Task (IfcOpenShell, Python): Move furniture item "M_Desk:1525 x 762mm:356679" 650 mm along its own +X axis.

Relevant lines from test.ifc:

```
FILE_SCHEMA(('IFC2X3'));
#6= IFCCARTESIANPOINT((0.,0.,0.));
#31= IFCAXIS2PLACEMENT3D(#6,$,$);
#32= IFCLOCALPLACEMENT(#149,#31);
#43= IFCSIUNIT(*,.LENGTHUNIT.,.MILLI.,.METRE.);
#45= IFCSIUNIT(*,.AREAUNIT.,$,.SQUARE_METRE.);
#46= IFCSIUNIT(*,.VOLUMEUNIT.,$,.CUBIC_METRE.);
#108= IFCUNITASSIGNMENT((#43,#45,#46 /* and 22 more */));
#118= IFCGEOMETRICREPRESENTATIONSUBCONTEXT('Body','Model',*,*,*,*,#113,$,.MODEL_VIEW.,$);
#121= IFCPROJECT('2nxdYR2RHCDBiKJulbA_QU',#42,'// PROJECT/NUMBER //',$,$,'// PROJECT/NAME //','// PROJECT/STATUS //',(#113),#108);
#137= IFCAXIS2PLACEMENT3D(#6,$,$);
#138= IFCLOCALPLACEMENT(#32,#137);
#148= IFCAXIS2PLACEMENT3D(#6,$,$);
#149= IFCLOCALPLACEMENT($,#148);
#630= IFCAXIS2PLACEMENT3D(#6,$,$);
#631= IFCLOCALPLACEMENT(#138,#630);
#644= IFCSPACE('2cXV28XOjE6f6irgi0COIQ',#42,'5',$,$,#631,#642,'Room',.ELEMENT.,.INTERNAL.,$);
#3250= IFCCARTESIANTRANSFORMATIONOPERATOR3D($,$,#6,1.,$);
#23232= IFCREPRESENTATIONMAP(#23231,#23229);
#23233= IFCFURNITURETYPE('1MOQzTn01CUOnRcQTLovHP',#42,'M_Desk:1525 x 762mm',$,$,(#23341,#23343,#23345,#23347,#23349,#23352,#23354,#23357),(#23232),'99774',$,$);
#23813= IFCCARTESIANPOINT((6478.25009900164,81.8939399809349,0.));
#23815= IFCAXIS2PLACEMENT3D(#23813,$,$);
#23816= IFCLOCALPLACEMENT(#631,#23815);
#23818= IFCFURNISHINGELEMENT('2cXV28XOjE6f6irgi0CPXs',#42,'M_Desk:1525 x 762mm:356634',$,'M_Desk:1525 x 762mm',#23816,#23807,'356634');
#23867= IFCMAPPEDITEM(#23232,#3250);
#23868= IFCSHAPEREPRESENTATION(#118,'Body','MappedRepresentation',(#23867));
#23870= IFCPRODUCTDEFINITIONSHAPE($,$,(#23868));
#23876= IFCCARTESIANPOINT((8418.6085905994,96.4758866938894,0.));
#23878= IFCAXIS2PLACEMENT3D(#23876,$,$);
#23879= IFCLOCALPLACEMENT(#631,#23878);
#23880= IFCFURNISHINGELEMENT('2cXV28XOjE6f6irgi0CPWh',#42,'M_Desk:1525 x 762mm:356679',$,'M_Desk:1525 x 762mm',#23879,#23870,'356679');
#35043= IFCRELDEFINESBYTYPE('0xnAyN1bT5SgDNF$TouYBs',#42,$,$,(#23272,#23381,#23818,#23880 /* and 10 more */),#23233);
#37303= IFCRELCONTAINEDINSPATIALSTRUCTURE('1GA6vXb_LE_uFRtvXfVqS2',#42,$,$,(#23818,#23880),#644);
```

```python
import ifcopenshell
import ifcopenshell.api.geometry
import ifcopenshell.util.placement
import ifcopenshell.util.unit

model = ifcopenshell.open("test.ifc")
unit_scale = ifcopenshell.util.unit.calculate_unit_scale(model)

item = model.by_guid("2cXV28XOjE6f6irgi0CPWh")
matrix = ifcopenshell.util.placement.get_local_placement(item.ObjectPlacement)
matrix[:3, 3] += matrix[:3, 0] * 0.65 / unit_scale
ifcopenshell.api.geometry.edit_object_placement(model, product=item, matrix=matrix, is_si=False)

print(ifcopenshell.util.placement.get_local_placement(item.ObjectPlacement).round(3) + 0.0)

model.write("test_updated.ifc")
```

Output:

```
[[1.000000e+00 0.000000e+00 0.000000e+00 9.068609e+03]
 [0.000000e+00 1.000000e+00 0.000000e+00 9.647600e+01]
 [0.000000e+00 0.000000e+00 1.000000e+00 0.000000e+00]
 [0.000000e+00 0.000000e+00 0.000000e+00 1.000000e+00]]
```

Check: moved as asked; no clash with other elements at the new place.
